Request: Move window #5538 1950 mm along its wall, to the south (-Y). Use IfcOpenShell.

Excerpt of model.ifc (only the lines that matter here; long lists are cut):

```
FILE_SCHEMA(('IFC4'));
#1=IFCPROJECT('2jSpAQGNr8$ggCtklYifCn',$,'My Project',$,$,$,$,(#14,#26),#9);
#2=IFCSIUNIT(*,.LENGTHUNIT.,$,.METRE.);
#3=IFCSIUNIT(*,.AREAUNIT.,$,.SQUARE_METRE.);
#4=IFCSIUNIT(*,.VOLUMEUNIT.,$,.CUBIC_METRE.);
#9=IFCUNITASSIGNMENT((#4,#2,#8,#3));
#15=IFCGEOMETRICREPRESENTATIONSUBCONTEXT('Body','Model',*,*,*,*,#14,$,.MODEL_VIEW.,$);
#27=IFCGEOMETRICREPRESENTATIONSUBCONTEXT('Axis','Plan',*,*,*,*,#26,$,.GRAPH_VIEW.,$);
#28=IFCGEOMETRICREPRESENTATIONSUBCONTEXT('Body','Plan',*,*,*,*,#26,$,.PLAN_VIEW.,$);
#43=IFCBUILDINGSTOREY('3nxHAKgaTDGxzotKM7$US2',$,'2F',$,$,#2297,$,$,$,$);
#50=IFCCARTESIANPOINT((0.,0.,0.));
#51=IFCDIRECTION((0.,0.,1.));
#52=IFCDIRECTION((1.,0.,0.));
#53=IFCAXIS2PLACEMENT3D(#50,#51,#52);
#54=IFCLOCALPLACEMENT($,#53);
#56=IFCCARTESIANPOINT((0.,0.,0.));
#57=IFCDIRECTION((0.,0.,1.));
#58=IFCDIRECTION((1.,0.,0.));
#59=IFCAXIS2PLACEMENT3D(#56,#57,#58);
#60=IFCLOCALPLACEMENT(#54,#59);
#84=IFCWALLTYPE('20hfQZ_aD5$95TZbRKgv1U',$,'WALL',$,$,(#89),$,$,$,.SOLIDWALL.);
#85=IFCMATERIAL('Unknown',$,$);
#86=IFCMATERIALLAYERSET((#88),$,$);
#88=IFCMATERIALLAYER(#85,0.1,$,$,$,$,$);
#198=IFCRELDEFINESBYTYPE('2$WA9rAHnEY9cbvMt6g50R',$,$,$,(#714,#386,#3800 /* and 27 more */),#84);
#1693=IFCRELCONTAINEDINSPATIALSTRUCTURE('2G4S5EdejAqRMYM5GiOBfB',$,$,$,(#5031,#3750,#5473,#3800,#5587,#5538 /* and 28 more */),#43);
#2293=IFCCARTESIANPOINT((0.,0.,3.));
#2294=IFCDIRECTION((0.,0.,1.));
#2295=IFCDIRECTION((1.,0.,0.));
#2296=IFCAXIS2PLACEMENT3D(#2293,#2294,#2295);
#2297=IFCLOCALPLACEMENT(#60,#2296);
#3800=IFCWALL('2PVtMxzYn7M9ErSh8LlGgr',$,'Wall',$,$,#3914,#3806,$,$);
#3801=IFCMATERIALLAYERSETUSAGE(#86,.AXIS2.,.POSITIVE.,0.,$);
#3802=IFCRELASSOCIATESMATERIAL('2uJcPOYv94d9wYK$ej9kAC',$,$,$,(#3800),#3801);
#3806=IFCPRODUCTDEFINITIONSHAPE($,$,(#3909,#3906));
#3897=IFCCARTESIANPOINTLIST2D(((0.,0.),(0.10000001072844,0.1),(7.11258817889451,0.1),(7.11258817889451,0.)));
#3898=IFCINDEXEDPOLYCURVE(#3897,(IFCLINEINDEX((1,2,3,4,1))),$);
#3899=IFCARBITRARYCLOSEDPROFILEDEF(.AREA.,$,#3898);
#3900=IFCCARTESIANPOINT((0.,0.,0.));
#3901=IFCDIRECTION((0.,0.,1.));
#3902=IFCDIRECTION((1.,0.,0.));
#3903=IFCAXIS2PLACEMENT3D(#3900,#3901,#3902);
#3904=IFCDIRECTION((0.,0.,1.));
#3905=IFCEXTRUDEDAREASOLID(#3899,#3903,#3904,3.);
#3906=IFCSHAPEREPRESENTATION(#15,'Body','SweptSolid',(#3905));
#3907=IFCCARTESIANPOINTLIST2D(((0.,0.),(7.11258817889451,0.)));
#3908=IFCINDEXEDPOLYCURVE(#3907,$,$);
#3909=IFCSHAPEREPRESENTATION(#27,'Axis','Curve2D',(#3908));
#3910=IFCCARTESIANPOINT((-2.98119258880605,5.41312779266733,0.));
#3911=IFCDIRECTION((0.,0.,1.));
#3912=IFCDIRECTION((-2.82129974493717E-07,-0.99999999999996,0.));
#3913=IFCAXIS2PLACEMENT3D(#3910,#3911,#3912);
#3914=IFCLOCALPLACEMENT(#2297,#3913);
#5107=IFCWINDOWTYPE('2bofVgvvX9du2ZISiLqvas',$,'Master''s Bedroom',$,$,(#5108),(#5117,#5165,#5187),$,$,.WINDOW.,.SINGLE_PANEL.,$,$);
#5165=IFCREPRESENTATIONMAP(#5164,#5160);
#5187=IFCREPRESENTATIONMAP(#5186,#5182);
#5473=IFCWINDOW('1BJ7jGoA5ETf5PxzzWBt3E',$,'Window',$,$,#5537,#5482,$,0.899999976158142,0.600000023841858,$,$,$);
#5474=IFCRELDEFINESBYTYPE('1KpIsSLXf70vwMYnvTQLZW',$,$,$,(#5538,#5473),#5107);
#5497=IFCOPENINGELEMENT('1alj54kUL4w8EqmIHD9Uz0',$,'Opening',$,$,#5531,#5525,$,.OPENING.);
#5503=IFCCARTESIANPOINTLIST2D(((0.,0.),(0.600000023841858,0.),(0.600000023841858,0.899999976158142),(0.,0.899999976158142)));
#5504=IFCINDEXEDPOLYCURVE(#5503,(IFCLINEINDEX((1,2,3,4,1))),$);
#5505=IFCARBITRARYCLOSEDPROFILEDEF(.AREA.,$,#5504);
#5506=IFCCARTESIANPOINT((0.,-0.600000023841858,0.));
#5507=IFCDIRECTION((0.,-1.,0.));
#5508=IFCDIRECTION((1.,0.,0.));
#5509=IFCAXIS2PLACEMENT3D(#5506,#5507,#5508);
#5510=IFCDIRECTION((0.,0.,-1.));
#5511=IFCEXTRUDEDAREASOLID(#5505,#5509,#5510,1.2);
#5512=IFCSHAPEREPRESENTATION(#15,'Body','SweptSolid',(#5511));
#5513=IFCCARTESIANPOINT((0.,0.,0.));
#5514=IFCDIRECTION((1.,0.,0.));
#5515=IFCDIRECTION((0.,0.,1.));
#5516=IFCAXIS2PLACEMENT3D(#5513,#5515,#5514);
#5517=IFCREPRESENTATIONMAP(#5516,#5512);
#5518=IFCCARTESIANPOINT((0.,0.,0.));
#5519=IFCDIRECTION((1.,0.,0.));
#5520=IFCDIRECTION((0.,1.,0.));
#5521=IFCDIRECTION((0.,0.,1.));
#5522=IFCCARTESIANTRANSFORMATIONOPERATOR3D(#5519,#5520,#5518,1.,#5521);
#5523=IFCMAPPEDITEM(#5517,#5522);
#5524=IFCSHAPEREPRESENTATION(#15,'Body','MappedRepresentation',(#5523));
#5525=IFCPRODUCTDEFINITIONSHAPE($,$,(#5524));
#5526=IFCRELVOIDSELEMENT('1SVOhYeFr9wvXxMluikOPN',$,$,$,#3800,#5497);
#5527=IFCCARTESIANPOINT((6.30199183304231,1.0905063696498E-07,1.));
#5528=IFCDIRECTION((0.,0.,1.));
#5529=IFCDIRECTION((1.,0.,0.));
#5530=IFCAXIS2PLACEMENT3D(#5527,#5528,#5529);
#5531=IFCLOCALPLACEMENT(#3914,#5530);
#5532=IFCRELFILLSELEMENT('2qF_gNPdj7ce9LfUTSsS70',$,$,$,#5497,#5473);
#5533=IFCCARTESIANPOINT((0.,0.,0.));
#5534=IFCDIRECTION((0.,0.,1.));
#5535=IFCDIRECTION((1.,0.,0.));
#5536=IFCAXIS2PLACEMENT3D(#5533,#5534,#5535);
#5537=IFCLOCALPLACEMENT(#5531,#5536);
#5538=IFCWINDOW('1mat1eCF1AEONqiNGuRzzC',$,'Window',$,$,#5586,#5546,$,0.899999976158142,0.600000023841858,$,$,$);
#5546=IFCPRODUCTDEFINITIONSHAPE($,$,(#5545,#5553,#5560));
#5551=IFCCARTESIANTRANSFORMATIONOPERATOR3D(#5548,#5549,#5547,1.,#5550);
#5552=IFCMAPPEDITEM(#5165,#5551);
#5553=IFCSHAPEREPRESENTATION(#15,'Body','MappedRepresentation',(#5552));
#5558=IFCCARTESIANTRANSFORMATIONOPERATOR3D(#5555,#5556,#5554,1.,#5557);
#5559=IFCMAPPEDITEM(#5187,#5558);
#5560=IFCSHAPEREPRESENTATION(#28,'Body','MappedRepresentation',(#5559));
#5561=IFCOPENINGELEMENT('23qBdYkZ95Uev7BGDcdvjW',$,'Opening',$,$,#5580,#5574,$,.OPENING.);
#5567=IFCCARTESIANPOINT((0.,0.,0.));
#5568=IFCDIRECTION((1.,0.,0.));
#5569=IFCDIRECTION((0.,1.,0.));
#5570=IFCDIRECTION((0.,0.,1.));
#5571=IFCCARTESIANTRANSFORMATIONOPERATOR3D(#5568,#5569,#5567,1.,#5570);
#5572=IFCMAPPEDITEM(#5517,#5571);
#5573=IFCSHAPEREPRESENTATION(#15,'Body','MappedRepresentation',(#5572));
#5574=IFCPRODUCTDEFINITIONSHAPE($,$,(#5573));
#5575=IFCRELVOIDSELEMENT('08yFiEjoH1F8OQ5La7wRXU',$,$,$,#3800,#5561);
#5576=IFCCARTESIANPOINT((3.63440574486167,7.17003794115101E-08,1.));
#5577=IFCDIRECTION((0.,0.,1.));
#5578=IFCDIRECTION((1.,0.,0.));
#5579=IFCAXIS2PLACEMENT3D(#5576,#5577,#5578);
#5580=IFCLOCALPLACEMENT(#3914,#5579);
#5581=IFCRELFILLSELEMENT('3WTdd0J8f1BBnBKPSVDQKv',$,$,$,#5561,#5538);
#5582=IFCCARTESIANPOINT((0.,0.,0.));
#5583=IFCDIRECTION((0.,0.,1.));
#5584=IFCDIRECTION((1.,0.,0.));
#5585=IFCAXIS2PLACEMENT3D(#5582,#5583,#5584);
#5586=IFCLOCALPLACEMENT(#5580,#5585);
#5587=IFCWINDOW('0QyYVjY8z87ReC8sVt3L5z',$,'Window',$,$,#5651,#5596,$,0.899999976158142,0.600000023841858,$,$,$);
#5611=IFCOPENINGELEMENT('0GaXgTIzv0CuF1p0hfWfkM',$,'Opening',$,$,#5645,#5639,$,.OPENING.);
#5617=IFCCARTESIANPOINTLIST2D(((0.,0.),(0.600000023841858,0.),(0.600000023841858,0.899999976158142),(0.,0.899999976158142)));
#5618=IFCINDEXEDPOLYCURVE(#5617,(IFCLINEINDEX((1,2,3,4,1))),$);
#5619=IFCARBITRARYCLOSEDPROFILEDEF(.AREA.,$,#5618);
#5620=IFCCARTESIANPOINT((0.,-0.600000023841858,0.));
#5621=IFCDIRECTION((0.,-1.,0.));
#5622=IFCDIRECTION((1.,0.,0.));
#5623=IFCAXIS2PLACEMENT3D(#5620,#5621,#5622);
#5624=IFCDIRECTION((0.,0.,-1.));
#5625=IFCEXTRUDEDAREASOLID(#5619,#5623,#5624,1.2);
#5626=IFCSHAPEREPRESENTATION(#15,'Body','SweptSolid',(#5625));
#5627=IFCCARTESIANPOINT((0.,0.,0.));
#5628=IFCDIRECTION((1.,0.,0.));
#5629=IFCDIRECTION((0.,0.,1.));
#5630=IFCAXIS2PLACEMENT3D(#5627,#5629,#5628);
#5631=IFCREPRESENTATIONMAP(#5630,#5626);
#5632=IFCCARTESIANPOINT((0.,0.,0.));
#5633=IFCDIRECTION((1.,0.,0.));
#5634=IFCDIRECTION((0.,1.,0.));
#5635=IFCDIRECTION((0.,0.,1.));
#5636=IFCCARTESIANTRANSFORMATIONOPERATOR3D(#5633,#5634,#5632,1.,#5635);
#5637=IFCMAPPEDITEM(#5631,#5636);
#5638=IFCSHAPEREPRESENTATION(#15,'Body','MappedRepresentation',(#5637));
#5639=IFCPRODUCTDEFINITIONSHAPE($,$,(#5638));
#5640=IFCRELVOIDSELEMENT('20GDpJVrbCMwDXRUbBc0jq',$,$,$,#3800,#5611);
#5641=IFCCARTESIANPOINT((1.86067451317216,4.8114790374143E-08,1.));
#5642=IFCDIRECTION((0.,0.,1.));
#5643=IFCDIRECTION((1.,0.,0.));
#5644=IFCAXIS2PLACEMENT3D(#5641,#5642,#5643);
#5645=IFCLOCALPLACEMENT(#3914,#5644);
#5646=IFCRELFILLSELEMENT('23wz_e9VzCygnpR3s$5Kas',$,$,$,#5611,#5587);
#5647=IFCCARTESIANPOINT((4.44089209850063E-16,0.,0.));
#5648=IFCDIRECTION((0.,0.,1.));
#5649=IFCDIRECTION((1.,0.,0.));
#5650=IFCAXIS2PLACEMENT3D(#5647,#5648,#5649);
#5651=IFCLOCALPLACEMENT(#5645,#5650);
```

```python
import ifcopenshell
import ifcopenshell.api.geometry
import ifcopenshell.util.placement
import ifcopenshell.util.unit

model = ifcopenshell.open("model.ifc")
unit_scale = ifcopenshell.util.unit.calculate_unit_scale(model)

window = model.by_guid("1mat1eCF1AEONqiNGuRzzC")
opening = window.FillsVoids[0].RelatingOpeningElement
wall = opening.VoidsElements[0].RelatingBuildingElement

wall_matrix = ifcopenshell.util.placement.get_local_placement(wall.ObjectPlacement)
shift = wall_matrix[:3, 0] * 1.95 / unit_scale
before = ifcopenshell.util.placement.get_local_placement(window.ObjectPlacement)[:3, 3].copy()

# The window is placed relative to its opening, so it follows when the opening moves.
matrix = ifcopenshell.util.placement.get_local_placement(opening.ObjectPlacement)
matrix[:3, 3] += shift
ifcopenshell.api.geometry.edit_object_placement(
    model, product=opening, matrix=matrix, is_si=False, should_transform_children=True
)

after = ifcopenshell.util.placement.get_local_placement(window.ObjectPlacement)[:3, 3]
print("window moved by", (after - before).round(3) + 0.0)

model.write("model_rev.ifc")
```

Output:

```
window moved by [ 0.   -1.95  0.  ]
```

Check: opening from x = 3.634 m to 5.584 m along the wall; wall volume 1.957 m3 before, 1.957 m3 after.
